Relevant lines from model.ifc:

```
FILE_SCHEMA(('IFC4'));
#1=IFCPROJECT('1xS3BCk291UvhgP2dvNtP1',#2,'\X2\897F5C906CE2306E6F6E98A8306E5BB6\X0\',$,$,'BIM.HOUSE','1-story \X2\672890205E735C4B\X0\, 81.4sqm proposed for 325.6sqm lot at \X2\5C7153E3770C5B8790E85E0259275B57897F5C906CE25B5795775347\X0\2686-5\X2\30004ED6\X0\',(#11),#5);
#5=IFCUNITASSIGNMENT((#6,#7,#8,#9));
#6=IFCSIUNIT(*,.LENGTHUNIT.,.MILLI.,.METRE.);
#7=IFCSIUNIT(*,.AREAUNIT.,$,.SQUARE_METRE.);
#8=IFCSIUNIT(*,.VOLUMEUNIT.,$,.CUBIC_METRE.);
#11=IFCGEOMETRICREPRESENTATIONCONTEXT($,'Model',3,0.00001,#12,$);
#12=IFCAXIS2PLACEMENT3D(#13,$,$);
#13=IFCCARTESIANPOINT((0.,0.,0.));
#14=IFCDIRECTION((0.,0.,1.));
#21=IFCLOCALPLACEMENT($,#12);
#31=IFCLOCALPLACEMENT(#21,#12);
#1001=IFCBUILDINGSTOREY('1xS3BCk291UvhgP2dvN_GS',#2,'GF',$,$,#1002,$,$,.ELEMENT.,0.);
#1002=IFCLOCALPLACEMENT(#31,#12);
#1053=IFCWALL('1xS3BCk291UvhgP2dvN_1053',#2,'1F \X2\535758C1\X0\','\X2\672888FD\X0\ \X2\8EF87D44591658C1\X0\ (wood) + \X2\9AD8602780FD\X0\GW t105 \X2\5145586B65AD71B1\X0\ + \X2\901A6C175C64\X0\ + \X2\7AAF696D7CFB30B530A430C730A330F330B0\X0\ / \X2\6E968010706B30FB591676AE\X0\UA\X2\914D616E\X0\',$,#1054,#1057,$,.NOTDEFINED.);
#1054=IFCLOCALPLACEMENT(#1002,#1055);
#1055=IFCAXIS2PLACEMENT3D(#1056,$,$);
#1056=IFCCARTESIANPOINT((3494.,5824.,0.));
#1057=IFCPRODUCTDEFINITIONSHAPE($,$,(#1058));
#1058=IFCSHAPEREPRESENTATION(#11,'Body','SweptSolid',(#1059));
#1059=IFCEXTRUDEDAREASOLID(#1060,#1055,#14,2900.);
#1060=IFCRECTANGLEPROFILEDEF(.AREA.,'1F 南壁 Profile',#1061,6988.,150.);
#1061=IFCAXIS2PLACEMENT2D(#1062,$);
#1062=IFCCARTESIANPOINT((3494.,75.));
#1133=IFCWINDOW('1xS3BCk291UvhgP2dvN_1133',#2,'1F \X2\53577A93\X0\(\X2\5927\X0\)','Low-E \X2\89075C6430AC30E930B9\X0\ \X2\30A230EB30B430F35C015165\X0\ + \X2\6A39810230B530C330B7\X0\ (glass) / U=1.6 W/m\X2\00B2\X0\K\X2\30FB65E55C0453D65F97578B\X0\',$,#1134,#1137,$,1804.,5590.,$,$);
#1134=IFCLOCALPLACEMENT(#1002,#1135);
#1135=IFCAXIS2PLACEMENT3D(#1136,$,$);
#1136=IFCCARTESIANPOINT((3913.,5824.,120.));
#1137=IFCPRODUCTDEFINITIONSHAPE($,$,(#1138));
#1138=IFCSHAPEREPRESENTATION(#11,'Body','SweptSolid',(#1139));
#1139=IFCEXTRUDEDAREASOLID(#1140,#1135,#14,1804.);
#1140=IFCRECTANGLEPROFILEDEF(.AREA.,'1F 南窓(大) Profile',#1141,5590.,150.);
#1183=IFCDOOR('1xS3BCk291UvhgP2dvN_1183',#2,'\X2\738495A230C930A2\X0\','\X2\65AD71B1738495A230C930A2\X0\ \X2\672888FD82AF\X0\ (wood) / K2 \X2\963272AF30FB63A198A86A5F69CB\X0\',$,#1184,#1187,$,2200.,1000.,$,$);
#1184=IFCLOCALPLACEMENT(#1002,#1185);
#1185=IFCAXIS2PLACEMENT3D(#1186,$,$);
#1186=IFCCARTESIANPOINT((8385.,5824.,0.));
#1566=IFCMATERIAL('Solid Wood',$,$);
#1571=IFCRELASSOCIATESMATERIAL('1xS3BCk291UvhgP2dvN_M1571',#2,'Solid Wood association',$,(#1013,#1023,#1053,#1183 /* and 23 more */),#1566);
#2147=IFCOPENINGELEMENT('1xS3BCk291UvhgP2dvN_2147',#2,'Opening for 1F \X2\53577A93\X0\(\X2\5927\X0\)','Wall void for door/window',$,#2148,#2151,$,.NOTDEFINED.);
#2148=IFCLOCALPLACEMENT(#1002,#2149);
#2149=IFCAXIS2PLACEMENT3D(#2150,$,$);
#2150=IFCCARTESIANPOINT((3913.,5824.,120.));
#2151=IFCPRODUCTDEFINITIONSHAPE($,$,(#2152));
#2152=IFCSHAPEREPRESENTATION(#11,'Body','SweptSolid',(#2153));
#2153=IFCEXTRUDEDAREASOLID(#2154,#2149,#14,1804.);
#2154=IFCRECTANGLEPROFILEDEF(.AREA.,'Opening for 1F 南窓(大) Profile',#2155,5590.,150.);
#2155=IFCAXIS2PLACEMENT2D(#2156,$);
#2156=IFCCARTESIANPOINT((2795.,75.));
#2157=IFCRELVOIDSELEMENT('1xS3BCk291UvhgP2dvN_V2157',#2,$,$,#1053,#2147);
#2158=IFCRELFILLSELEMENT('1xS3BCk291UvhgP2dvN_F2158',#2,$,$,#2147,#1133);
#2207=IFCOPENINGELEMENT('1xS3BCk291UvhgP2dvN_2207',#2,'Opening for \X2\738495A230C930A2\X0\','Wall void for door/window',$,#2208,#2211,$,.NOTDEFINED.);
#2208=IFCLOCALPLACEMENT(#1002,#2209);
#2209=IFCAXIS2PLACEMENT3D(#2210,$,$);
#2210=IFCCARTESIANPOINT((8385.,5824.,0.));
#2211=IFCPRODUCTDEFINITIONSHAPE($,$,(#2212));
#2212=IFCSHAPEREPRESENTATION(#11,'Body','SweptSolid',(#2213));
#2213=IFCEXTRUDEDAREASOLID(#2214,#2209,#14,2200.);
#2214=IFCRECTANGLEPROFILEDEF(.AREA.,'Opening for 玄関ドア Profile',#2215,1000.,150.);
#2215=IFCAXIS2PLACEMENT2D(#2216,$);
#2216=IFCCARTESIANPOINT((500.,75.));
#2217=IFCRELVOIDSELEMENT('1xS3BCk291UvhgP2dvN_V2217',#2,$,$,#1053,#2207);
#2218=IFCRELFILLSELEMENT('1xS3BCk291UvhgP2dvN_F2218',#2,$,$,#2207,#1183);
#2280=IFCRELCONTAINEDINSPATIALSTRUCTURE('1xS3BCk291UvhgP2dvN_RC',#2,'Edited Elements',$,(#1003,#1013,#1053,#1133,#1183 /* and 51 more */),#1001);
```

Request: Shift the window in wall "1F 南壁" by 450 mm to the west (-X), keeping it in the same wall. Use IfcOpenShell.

```python
import ifcopenshell
import ifcopenshell.api.geometry
import ifcopenshell.util.placement

model = ifcopenshell.open("model.ifc")

window = model.by_guid("1xS3BCk291UvhgP2dvN_1133")
opening = window.FillsVoids[0].RelatingOpeningElement
wall = opening.VoidsElements[0].RelatingBuildingElement

wall_matrix = ifcopenshell.util.placement.get_local_placement(wall.ObjectPlacement)
shift = wall_matrix[:3, 0] * -450.0
before = ifcopenshell.util.placement.get_local_placement(window.ObjectPlacement)[:3, 3].copy()

# The window is not placed relative to its opening, so move both.
for product in (opening, window):
    matrix = ifcopenshell.util.placement.get_local_placement(product.ObjectPlacement)
    matrix[:3, 3] += shift
    ifcopenshell.api.geometry.edit_object_placement(model, product=product, matrix=matrix, is_si=False)

after = ifcopenshell.util.placement.get_local_placement(window.ObjectPlacement)[:3, 3]
print("window moved by", (after - before).round(3) + 0.0)

model.write("model_updated.ifc")
```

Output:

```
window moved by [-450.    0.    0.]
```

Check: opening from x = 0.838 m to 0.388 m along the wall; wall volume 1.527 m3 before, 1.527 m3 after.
